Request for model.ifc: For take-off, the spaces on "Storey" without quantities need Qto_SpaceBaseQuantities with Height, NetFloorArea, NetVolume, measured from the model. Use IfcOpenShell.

First a look at what the model holds.

```python
import ifcopenshell
import ifcopenshell.util.element
import ifcopenshell.util.unit

model = ifcopenshell.open("model.ifc")
print(model.schema)
for unit_type in ("LENGTHUNIT", "AREAUNIT", "VOLUMEUNIT"):
    print(unit_type, ifcopenshell.util.unit.calculate_unit_scale(model, unit_type))
storey = next(s for s in model.by_type("IfcBuildingStorey") if s.Name == "Storey")
spaces = [e for e in ifcopenshell.util.element.get_decomposition(storey) if e.is_a("IfcSpace")]
for e in sorted(spaces, key=lambda e: e.id()):
    print(e.id(), e.is_a(), e.Name, list(ifcopenshell.util.element.get_psets(e, qtos_only=True)), sep=" | ")
```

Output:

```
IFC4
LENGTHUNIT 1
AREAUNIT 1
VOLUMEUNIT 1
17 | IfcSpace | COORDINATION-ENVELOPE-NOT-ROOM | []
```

```python
import ifcopenshell
import ifcopenshell.api.pset
import ifcopenshell.geom
import ifcopenshell.util.element
import ifcopenshell.util.shape
import ifcopenshell.util.unit

model = ifcopenshell.open("model.ifc")
unit_scale = ifcopenshell.util.unit.calculate_unit_scale(model)
area_scale = ifcopenshell.util.unit.calculate_unit_scale(model, "AREAUNIT")
volume_scale = ifcopenshell.util.unit.calculate_unit_scale(model, "VOLUMEUNIT")
settings = ifcopenshell.geom.settings()

storey = next(s for s in model.by_type("IfcBuildingStorey") if s.Name == "Storey")
spaces = [e for e in ifcopenshell.util.element.get_decomposition(storey) if e.is_a("IfcSpace")]

for e in sorted(spaces, key=lambda e: e.id()):
    if ifcopenshell.util.element.get_psets(e, qtos_only=True, should_inherit=False):
        continue
    # Geometry comes back in metres, in the element's own axes.
    shape = ifcopenshell.geom.create_shape(settings, e)
    values = {
        "Height": ifcopenshell.util.shape.get_z(shape.geometry) / unit_scale,
        "NetFloorArea": ifcopenshell.util.shape.get_footprint_area(shape.geometry) / area_scale,
        "NetVolume": ifcopenshell.util.shape.get_volume(shape.geometry) / volume_scale,
    }
    qto = ifcopenshell.api.pset.add_qto(model, product=e, name="Qto_SpaceBaseQuantities")
    ifcopenshell.api.pset.edit_qto(model, qto=qto, properties=values)
    print(e.id(), {k: round(v, 3) for k, v in values.items()})

model.write("model-out.ifc")
```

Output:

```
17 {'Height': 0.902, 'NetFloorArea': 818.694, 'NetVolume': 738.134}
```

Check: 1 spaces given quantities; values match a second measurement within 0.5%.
